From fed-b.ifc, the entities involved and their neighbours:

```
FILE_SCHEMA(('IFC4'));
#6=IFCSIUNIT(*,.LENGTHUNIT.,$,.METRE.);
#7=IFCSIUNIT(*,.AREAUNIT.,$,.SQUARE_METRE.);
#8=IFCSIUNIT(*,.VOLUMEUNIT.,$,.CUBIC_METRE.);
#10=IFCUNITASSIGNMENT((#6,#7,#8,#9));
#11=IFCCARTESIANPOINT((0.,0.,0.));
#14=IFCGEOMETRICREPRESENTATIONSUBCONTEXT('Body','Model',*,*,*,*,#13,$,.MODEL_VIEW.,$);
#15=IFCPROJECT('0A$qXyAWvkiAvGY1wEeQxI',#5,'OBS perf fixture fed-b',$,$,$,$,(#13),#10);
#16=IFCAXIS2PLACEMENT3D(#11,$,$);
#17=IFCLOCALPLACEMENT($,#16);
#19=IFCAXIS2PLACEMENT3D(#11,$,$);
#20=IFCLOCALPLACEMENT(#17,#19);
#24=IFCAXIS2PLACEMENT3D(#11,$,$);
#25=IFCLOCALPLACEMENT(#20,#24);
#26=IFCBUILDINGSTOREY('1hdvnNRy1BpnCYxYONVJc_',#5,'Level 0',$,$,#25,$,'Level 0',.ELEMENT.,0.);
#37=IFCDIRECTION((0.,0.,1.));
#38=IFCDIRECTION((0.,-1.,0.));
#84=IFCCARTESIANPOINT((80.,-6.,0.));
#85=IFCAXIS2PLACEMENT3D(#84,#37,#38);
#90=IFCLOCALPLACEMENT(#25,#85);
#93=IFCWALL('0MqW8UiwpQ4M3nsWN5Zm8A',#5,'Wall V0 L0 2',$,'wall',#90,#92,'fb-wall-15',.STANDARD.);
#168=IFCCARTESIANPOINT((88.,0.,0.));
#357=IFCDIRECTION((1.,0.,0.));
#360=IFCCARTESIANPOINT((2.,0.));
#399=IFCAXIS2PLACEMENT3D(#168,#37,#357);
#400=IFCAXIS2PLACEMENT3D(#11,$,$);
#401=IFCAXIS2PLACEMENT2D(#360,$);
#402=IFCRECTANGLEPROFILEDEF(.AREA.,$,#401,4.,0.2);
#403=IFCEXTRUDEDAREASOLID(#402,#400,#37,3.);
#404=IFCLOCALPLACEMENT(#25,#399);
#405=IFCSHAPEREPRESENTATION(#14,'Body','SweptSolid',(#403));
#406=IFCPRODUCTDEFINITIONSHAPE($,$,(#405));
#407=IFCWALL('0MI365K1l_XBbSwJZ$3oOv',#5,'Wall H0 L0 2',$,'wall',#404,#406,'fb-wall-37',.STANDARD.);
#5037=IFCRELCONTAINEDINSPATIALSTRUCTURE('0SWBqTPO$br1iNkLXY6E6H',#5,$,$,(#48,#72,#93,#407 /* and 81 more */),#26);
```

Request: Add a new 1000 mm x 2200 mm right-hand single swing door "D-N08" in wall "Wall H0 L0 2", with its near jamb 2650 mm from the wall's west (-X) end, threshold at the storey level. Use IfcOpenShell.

```python
import numpy as np
import ifcopenshell
import ifcopenshell.api.feature
import ifcopenshell.api.geometry
import ifcopenshell.api.root
import ifcopenshell.api.spatial
import ifcopenshell.geom
import ifcopenshell.util.element
import ifcopenshell.util.placement
import ifcopenshell.util.representation
import ifcopenshell.util.shape
import ifcopenshell.util.unit

model = ifcopenshell.open("fed-b.ifc")
unit_scale = ifcopenshell.util.unit.calculate_unit_scale(model)
settings = ifcopenshell.geom.settings()


def volume(element):
    """Net volume in cubic metres, openings subtracted."""
    shape = ifcopenshell.geom.create_shape(settings, element)
    return ifcopenshell.util.shape.get_volume(shape.geometry)


wall = model.by_id(407)
storey = ifcopenshell.util.element.get_container(wall, ifc_class="IfcBuildingStorey")
context = ifcopenshell.util.representation.get_context(model, "Model", "Body", "MODEL_VIEW")
before = volume(wall)

width, height, from_end, sill = 1, 2.2, 2.65, 0.0  # metres

# The wall runs along its own X axis, and the end named is its -X end.
wall_shape = ifcopenshell.geom.create_shape(settings, wall)
x, y, z = ifcopenshell.util.shape.get_vertices(wall_shape.geometry).T
start = x.min() + from_end
face, thickness = float(y.min()), float(y.max() - y.min())
wall_matrix = ifcopenshell.util.placement.get_local_placement(wall.ObjectPlacement)
level = ifcopenshell.util.placement.get_local_placement(storey.ObjectPlacement)[2, 3]


def in_wall(x, y):
    """Placement at x, y metres in the wall's axes, at sill height."""
    matrix = wall_matrix.copy()
    matrix[:, 3] = wall_matrix @ np.array([x / unit_scale, y / unit_scale, 0.0, 1.0])
    matrix[2, 3] = level + sill / unit_scale
    return matrix


# Opening: a box that overshoots both wall faces by 50 mm.
opening = ifcopenshell.api.root.create_entity(model, ifc_class="IfcOpeningElement", predefined_type="OPENING")
box = ifcopenshell.api.geometry.add_wall_representation(
    model, context=context, length=width, height=height, thickness=thickness + 0.1
)
ifcopenshell.api.geometry.assign_representation(model, product=opening, representation=box)
ifcopenshell.api.geometry.edit_object_placement(model, product=opening, matrix=in_wall(start, face - 0.05), is_si=False)
ifcopenshell.api.feature.add_feature(model, feature=opening, element=wall)

door = ifcopenshell.api.root.create_entity(model, ifc_class="IfcDoor", name="D-N08", predefined_type="DOOR")
door.OverallWidth, door.OverallHeight = width / unit_scale, height / unit_scale
door.OperationType = "SINGLE_SWING_RIGHT"
body = ifcopenshell.api.geometry.add_door_representation(
    model,
    context=context,
    overall_width=door.OverallWidth,
    overall_height=door.OverallHeight,
    operation_type="SINGLE_SWING_RIGHT",
    lining_properties={"LiningDepth": thickness / unit_scale, "ThresholdDepth": thickness / unit_scale},
)
ifcopenshell.api.geometry.assign_representation(model, product=door, representation=body)
ifcopenshell.api.spatial.assign_container(model, products=[door], relating_structure=storey)
ifcopenshell.api.feature.add_filling(model, opening=opening, element=door)

# The lining spans the wall, so the door starts at the wall face.
ifcopenshell.api.geometry.edit_object_placement(model, product=door, matrix=in_wall(start, face), is_si=False)

after = volume(wall)

print(f"wall volume {before:.3f} -> {after:.3f} m3")

model.write("fed-b-out.ifc")
```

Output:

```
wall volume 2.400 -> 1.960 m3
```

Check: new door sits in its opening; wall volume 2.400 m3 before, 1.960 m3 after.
